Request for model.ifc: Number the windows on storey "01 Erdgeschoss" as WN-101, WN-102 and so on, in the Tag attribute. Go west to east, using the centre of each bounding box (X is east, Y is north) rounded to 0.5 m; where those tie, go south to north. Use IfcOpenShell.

First a look at what the model holds.

```python
import ifcopenshell
import ifcopenshell.util.element
import ifcopenshell.util.placement

model = ifcopenshell.open("model.ifc")
print(model.schema)
storey = next(s for s in model.by_type("IfcBuildingStorey") if s.Name == "01 Erdgeschoss")
windows = [e for e in ifcopenshell.util.element.get_decomposition(storey) if e.is_a("IfcWindow")]
for e in sorted(windows, key=lambda e: e.id()):
    origin = ifcopenshell.util.placement.get_local_placement(e.ObjectPlacement)[:3, 3]
    print(e.id(), e.Tag, e.Name, origin.round(2) + 0.0, sep=" | ")
```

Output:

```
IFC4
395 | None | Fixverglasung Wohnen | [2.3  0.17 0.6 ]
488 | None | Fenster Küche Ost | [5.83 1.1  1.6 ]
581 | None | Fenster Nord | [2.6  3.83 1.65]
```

```python
import ifcopenshell
import ifcopenshell.geom
import ifcopenshell.util.element
import ifcopenshell.util.shape

model = ifcopenshell.open("model.ifc")
settings = ifcopenshell.geom.settings()
settings.set("use-world-coords", True)


def centre(element):
    shape = ifcopenshell.geom.create_shape(settings, element)
    return ifcopenshell.util.shape.get_bbox_centroid(shape.geometry)


storey = next(s for s in model.by_type("IfcBuildingStorey") if s.Name == "01 Erdgeschoss")
windows = [e for e in ifcopenshell.util.element.get_decomposition(storey) if e.is_a("IfcWindow")]

# Insertion points can sit at a corner or the storey origin, so sort by the geometry (in metres).
centres = {e: centre(e) for e in windows}
windows.sort(key=lambda e: (round(centres[e][0] / 0.5), centres[e][1]))

for i, e in enumerate(windows, start=1):
    number = f"WN-1{i:02d}"
    e.Tag = number
    print(e.id(), number)

model.write("model_edited.ifc")
```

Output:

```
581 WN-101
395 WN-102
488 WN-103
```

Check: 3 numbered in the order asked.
